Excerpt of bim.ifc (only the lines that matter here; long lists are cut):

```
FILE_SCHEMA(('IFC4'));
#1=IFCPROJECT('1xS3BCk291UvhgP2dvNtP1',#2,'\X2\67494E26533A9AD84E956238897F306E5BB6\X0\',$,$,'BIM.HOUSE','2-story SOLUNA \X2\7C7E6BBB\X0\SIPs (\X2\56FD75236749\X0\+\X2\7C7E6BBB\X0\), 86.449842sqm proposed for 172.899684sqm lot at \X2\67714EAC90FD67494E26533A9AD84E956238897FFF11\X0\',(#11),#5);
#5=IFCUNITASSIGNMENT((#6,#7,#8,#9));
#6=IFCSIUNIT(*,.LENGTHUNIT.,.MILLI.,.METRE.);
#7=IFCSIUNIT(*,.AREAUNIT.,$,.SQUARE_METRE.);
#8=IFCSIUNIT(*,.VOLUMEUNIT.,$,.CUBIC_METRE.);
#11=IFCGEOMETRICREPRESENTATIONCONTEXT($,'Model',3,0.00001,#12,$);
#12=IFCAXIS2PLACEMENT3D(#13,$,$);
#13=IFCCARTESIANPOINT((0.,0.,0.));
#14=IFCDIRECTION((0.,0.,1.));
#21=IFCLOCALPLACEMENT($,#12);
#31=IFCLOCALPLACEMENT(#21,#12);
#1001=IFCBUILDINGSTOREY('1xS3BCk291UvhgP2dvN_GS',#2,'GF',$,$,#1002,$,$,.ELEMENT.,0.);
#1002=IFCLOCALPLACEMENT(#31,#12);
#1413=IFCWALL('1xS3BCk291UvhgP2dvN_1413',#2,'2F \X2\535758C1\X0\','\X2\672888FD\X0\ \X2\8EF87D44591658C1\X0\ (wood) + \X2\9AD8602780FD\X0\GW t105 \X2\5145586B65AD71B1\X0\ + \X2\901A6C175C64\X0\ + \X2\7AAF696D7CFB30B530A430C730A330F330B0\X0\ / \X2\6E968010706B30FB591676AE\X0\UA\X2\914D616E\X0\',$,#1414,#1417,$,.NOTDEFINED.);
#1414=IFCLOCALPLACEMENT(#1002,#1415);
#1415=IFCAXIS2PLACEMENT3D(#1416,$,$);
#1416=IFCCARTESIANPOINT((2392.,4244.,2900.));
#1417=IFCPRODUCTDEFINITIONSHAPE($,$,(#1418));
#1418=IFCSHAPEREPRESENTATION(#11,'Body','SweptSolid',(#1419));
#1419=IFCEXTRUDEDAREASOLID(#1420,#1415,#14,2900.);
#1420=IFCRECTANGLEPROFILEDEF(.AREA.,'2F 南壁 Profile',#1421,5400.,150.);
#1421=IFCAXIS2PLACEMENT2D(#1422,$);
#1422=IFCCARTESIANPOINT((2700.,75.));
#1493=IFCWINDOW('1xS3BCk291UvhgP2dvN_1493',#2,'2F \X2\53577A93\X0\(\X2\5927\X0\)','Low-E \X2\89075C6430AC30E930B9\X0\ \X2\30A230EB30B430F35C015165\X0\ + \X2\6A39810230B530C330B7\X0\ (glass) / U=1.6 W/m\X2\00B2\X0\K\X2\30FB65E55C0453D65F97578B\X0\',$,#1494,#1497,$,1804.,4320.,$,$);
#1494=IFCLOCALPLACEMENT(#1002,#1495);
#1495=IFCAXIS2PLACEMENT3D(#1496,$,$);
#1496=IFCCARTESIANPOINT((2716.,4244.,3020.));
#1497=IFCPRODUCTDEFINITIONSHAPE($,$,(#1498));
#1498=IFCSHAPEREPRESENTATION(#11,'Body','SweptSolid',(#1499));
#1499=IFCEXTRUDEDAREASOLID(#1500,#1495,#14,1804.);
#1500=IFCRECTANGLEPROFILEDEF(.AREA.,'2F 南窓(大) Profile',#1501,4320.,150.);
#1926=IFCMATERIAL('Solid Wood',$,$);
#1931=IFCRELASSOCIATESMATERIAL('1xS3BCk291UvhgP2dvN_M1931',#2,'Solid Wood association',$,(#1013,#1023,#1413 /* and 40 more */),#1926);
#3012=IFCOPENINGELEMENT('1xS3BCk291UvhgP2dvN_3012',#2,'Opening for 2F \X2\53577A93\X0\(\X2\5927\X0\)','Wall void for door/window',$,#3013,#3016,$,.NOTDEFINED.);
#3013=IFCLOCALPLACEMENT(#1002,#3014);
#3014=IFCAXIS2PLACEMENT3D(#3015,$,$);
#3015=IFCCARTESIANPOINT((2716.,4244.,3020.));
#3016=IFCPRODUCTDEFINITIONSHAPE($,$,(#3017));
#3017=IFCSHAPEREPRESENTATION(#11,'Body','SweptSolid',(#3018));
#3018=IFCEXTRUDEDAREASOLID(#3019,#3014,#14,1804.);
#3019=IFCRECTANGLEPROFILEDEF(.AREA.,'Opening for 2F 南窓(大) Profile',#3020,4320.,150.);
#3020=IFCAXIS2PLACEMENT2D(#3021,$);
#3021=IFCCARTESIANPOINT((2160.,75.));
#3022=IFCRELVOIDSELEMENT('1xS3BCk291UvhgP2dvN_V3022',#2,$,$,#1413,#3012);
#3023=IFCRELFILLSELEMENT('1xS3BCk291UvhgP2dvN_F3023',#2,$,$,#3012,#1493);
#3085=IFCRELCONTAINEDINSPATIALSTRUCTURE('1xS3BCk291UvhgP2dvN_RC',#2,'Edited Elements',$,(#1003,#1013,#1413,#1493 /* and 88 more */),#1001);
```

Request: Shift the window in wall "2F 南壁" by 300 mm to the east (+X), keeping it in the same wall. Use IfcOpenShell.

```python
import ifcopenshell
import ifcopenshell.api.geometry
import ifcopenshell.util.placement
import ifcopenshell.util.unit

model = ifcopenshell.open("bim.ifc")
unit_scale = ifcopenshell.util.unit.calculate_unit_scale(model)

window = model.by_guid("1xS3BCk291UvhgP2dvN_1493")
opening = window.FillsVoids[0].RelatingOpeningElement
wall = opening.VoidsElements[0].RelatingBuildingElement

wall_matrix = ifcopenshell.util.placement.get_local_placement(wall.ObjectPlacement)
shift = wall_matrix[:3, 0] * 0.3 / unit_scale
before = ifcopenshell.util.placement.get_local_placement(window.ObjectPlacement)[:3, 3].copy()

# The window is not placed relative to its opening, so move both.
for product in (opening, window):
    matrix = ifcopenshell.util.placement.get_local_placement(product.ObjectPlacement)
    matrix[:3, 3] += shift
    ifcopenshell.api.geometry.edit_object_placement(model, product=product, matrix=matrix, is_si=False)

after = ifcopenshell.util.placement.get_local_placement(window.ObjectPlacement)[:3, 3]
print("window moved by", (after - before).round(3) + 0.0)

model.write("bim_rev.ifc")
```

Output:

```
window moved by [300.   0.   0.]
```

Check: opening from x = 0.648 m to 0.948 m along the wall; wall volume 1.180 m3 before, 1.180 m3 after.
